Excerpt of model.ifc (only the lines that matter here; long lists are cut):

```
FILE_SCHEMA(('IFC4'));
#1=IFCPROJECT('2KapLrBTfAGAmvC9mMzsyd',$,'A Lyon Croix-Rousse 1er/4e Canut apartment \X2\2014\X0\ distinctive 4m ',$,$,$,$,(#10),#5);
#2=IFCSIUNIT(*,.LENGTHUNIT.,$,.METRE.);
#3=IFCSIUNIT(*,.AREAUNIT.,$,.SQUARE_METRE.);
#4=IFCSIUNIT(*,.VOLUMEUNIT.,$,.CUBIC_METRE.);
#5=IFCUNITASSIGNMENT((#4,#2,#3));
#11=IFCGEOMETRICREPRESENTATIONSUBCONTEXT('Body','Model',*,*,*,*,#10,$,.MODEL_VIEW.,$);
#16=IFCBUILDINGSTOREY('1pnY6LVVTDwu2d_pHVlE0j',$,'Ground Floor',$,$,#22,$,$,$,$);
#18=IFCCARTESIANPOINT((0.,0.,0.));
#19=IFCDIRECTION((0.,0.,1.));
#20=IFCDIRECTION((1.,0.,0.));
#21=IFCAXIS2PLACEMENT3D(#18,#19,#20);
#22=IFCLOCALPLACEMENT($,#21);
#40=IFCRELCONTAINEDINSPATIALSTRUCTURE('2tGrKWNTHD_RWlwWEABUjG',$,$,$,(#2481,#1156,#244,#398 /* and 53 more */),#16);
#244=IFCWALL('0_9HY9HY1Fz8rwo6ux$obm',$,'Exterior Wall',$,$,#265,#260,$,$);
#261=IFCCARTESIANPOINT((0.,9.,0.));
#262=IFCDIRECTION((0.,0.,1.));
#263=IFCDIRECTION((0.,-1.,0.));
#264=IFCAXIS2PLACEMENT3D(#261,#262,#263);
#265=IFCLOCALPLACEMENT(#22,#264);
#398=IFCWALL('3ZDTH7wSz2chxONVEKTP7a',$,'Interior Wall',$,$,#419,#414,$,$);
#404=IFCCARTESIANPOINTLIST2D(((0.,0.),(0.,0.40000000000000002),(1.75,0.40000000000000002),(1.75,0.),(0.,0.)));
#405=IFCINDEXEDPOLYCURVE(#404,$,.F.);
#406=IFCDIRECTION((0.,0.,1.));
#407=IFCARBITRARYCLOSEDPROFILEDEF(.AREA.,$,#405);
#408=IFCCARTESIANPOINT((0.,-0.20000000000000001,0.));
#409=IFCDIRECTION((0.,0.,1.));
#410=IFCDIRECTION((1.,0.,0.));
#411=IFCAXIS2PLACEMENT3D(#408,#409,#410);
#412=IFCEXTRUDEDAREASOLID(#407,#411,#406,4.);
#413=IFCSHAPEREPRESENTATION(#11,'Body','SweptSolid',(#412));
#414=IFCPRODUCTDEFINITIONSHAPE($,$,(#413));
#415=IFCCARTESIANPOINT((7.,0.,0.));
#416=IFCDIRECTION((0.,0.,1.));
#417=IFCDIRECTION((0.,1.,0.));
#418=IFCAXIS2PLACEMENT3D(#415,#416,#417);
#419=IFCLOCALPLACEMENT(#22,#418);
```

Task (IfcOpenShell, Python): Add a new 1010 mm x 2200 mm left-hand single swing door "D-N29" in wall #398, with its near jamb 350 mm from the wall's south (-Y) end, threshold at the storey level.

```python
import numpy as np
import ifcopenshell
import ifcopenshell.api.feature
import ifcopenshell.api.geometry
import ifcopenshell.api.root
import ifcopenshell.api.spatial
import ifcopenshell.geom
import ifcopenshell.util.element
import ifcopenshell.util.placement
import ifcopenshell.util.representation
import ifcopenshell.util.shape
import ifcopenshell.util.unit

model = ifcopenshell.open("model.ifc")
unit_scale = ifcopenshell.util.unit.calculate_unit_scale(model)
settings = ifcopenshell.geom.settings()


def volume(element):
    """Net volume in cubic metres, openings subtracted."""
    shape = ifcopenshell.geom.create_shape(settings, element)
    return ifcopenshell.util.shape.get_volume(shape.geometry)


wall = model.by_guid("3ZDTH7wSz2chxONVEKTP7a")
storey = ifcopenshell.util.element.get_container(wall, ifc_class="IfcBuildingStorey")
context = ifcopenshell.util.representation.get_context(model, "Model", "Body", "MODEL_VIEW")
before = volume(wall)

width, height, from_end, sill = 1.01, 2.2, 0.35, 0.0  # metres

# The wall runs along its own X axis, and the end named is its -X end.
wall_shape = ifcopenshell.geom.create_shape(settings, wall)
x, y, z = ifcopenshell.util.shape.get_vertices(wall_shape.geometry).T
start = x.min() + from_end
face, thickness = float(y.min()), float(y.max() - y.min())
wall_matrix = ifcopenshell.util.placement.get_local_placement(wall.ObjectPlacement)
level = ifcopenshell.util.placement.get_local_placement(storey.ObjectPlacement)[2, 3]


def in_wall(x, y):
    """Placement at x, y metres in the wall's axes, at sill height."""
    matrix = wall_matrix.copy()
    matrix[:, 3] = wall_matrix @ np.array([x / unit_scale, y / unit_scale, 0.0, 1.0])
    matrix[2, 3] = level + sill / unit_scale
    return matrix


# Opening: a box that overshoots both wall faces by 50 mm.
opening = ifcopenshell.api.root.create_entity(model, ifc_class="IfcOpeningElement", predefined_type="OPENING")
box = ifcopenshell.api.geometry.add_wall_representation(
    model, context=context, length=width, height=height, thickness=thickness + 0.1
)
ifcopenshell.api.geometry.assign_representation(model, product=opening, representation=box)
ifcopenshell.api.geometry.edit_object_placement(model, product=opening, matrix=in_wall(start, face - 0.05), is_si=False)
ifcopenshell.api.feature.add_feature(model, feature=opening, element=wall)

door = ifcopenshell.api.root.create_entity(model, ifc_class="IfcDoor", name="D-N29", predefined_type="DOOR")
door.OverallWidth, door.OverallHeight = width / unit_scale, height / unit_scale
door.OperationType = "SINGLE_SWING_LEFT"
body = ifcopenshell.api.geometry.add_door_representation(
    model,
    context=context,
    overall_width=door.OverallWidth,
    overall_height=door.OverallHeight,
    operation_type="SINGLE_SWING_LEFT",
    lining_properties={"LiningDepth": thickness / unit_scale, "ThresholdDepth": thickness / unit_scale},
)
ifcopenshell.api.geometry.assign_representation(model, product=door, representation=body)
ifcopenshell.api.spatial.assign_container(model, products=[door], relating_structure=storey)
ifcopenshell.api.feature.add_filling(model, opening=opening, element=door)

# The lining spans the wall, so the door starts at the wall face.
ifcopenshell.api.geometry.edit_object_placement(model, product=door, matrix=in_wall(start, face), is_si=False)

after = volume(wall)

print(f"wall volume {before:.3f} -> {after:.3f} m3")

model.write("model-out.ifc")
```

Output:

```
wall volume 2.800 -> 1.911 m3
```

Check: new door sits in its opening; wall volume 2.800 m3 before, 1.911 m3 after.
